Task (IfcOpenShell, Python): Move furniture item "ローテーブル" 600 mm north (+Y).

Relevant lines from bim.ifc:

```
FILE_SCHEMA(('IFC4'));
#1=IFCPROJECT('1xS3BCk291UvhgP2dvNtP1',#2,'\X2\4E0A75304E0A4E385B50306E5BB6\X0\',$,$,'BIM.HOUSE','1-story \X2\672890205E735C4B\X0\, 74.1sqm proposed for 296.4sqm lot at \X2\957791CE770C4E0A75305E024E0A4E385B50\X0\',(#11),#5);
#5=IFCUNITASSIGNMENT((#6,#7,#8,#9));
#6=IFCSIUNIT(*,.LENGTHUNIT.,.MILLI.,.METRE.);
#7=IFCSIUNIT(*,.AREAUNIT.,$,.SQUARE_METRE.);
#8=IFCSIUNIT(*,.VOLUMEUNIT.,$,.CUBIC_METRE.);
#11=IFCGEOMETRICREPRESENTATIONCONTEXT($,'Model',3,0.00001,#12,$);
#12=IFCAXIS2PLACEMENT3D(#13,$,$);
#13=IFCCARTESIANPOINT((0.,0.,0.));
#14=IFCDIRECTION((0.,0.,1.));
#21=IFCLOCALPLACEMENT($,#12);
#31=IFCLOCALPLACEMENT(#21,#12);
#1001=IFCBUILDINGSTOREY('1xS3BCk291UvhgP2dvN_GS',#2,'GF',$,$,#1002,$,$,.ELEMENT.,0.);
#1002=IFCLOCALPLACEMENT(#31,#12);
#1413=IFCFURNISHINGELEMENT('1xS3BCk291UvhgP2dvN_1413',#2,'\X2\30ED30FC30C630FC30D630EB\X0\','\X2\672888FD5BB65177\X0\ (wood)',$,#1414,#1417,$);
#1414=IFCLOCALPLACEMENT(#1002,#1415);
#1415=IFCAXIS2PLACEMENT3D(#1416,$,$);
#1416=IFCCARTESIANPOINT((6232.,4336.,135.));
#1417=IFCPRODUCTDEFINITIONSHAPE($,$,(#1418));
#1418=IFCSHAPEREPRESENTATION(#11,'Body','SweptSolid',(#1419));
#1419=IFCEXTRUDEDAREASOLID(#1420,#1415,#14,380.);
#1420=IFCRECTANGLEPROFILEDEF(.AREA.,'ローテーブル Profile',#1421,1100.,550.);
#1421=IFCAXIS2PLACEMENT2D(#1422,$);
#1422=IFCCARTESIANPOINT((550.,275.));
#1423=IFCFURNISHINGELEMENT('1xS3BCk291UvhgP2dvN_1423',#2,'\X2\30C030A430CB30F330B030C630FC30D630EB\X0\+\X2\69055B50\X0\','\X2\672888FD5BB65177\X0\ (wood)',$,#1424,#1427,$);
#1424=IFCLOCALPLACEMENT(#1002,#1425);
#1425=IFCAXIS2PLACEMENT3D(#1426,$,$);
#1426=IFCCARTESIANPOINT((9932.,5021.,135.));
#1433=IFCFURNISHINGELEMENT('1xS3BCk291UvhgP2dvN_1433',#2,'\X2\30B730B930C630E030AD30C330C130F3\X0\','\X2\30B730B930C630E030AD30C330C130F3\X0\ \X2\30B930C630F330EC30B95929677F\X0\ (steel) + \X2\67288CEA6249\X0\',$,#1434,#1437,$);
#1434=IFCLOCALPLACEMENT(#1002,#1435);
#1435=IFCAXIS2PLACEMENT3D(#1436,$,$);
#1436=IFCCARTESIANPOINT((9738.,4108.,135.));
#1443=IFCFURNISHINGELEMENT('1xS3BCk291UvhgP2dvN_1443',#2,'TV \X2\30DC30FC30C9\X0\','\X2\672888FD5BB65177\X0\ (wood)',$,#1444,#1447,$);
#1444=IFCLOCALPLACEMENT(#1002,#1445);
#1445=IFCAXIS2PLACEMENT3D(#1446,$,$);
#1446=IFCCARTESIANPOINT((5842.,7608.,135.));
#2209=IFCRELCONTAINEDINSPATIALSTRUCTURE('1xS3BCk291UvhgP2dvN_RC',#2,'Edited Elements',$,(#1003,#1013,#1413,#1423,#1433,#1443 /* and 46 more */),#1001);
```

```python
import ifcopenshell
import ifcopenshell.api.geometry
import ifcopenshell.util.placement
import ifcopenshell.util.unit

model = ifcopenshell.open("bim.ifc")
unit_scale = ifcopenshell.util.unit.calculate_unit_scale(model)

item = model.by_guid("1xS3BCk291UvhgP2dvN_1413")
matrix = ifcopenshell.util.placement.get_local_placement(item.ObjectPlacement)
matrix[1, 3] += 0.6 / unit_scale
ifcopenshell.api.geometry.edit_object_placement(model, product=item, matrix=matrix, is_si=False)

print(ifcopenshell.util.placement.get_local_placement(item.ObjectPlacement).round(3) + 0.0)

model.write("bim-out.ifc")
```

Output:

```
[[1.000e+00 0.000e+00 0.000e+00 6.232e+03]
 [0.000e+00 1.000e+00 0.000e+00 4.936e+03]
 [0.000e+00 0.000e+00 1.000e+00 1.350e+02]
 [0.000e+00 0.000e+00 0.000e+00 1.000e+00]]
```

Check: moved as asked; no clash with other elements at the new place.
